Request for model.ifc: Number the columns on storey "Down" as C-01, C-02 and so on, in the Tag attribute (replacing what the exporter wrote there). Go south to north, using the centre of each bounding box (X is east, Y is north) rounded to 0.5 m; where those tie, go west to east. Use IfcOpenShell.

First a look at what the model holds.

```python
import ifcopenshell
import ifcopenshell.util.element
import ifcopenshell.util.placement

model = ifcopenshell.open("model.ifc")
print(model.schema)
storey = next(s for s in model.by_type("IfcBuildingStorey") if s.Name == "Down")
columns = [e for e in ifcopenshell.util.element.get_decomposition(storey) if e.is_a("IfcColumn")]
for e in sorted(columns, key=lambda e: e.id()):
    origin = ifcopenshell.util.placement.get_local_placement(e.ObjectPlacement)[:3, 3]
    print(e.id(), e.Tag, e.Name, origin.round(2) + 0.0, sep=" | ")
```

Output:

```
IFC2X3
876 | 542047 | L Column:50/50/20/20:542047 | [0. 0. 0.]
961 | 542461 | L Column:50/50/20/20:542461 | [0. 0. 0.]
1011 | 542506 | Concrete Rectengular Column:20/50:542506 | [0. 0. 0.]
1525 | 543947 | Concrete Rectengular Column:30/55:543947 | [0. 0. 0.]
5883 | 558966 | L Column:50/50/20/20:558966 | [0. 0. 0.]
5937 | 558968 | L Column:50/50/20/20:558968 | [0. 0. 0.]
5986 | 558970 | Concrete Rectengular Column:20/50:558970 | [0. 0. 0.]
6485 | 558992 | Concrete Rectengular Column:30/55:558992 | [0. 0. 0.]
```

```python
import ifcopenshell
import ifcopenshell.geom
import ifcopenshell.util.element
import ifcopenshell.util.shape

model = ifcopenshell.open("model.ifc")
settings = ifcopenshell.geom.settings()
settings.set("use-world-coords", True)


def centre(element):
    shape = ifcopenshell.geom.create_shape(settings, element)
    return ifcopenshell.util.shape.get_bbox_centroid(shape.geometry)


storey = next(s for s in model.by_type("IfcBuildingStorey") if s.Name == "Down")
columns = [e for e in ifcopenshell.util.element.get_decomposition(storey) if e.is_a("IfcColumn")]

# Insertion points can sit at a corner or the storey origin, so sort by the geometry (in metres).
centres = {e: centre(e) for e in columns}
columns.sort(key=lambda e: (round(centres[e][1] / 0.5), centres[e][0]))

for i, e in enumerate(columns, start=1):
    number = f"C-{i:02d}"
    e.Tag = number
    print(e.id(), number)

model.write("model-out.ifc")
```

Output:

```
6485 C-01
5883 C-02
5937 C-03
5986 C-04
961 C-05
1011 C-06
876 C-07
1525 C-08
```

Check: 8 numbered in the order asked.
